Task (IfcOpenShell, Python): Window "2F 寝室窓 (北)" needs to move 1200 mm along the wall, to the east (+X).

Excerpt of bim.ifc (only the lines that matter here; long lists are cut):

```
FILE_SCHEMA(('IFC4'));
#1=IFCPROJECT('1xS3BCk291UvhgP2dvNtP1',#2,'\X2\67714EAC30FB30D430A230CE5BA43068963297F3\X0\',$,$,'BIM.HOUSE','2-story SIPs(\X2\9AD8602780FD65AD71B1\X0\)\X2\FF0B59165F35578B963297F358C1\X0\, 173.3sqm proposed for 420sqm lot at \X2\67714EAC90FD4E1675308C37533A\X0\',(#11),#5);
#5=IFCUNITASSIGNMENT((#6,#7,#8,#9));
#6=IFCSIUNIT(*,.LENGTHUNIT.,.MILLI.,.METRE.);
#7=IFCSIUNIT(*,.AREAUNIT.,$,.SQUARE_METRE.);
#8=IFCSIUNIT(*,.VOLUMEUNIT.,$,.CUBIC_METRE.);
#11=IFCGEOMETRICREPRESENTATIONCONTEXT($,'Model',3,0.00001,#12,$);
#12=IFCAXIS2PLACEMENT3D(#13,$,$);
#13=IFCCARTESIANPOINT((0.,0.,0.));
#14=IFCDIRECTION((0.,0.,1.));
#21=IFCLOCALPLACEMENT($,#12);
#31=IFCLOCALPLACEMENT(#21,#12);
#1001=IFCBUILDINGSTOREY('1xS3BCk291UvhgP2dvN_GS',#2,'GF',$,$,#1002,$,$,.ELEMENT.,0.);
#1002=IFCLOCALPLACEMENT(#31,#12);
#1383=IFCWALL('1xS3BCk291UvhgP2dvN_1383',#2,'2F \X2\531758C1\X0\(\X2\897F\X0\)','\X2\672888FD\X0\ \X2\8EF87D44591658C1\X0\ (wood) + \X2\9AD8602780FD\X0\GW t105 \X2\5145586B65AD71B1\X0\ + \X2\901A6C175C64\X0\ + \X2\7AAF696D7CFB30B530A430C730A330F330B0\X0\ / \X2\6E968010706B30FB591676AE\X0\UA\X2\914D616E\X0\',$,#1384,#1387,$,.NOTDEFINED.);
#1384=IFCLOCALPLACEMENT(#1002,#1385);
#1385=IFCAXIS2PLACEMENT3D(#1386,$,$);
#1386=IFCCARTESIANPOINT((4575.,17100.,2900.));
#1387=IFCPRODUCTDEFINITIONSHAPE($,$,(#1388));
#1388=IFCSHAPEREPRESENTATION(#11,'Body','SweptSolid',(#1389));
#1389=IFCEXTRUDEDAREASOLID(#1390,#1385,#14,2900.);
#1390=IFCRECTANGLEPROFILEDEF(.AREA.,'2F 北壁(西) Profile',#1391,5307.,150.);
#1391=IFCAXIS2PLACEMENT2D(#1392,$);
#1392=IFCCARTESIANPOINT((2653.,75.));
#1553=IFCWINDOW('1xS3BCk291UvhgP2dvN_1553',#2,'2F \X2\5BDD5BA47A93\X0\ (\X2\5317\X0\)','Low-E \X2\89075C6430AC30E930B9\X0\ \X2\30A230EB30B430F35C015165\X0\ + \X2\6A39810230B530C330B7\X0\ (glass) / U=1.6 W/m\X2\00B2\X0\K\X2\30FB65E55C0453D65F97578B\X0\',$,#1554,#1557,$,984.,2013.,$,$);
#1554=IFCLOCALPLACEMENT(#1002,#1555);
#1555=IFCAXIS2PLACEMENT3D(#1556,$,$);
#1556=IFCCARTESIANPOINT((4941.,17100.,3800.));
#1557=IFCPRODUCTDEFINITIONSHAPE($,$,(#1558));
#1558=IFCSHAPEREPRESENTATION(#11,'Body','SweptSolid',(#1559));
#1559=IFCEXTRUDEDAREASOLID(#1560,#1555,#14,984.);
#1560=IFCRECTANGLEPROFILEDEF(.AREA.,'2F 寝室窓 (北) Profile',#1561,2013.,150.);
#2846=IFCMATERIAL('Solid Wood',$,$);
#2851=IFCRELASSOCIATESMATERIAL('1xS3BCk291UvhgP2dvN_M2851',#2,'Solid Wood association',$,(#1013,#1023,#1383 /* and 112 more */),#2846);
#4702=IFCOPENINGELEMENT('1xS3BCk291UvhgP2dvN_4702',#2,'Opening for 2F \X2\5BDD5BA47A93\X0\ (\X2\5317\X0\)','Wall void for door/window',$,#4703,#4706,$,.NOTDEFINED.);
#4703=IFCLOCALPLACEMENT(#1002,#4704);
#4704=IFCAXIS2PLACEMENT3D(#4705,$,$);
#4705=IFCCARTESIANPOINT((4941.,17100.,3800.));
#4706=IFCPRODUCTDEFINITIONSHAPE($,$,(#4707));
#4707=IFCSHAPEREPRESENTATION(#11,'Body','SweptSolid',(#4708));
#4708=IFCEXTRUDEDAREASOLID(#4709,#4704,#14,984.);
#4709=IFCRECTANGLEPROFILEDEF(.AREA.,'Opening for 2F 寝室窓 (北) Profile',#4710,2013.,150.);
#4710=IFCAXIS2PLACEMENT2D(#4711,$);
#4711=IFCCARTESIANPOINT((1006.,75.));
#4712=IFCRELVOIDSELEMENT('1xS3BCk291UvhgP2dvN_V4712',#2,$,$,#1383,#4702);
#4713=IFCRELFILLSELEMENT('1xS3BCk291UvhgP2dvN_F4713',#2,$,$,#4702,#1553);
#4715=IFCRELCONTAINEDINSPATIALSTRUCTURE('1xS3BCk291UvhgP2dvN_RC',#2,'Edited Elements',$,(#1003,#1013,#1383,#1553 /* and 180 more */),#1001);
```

```python
import ifcopenshell
import ifcopenshell.api.geometry
import ifcopenshell.util.placement
import ifcopenshell.util.unit

model = ifcopenshell.open("bim.ifc")
unit_scale = ifcopenshell.util.unit.calculate_unit_scale(model)

window = model.by_id(1553)
opening = window.FillsVoids[0].RelatingOpeningElement
wall = opening.VoidsElements[0].RelatingBuildingElement

wall_matrix = ifcopenshell.util.placement.get_local_placement(wall.ObjectPlacement)
shift = wall_matrix[:3, 0] * 1.2 / unit_scale
before = ifcopenshell.util.placement.get_local_placement(window.ObjectPlacement)[:3, 3].copy()

# The window is not placed relative to its opening, so move both.
for product in (opening, window):
    matrix = ifcopenshell.util.placement.get_local_placement(product.ObjectPlacement)
    matrix[:3, 3] += shift
    ifcopenshell.api.geometry.edit_object_placement(model, product=product, matrix=matrix, is_si=False)

after = ifcopenshell.util.placement.get_local_placement(window.ObjectPlacement)[:3, 3]
print("window moved by", (after - before).round(3) + 0.0)

model.write("bim_rev.ifc")
```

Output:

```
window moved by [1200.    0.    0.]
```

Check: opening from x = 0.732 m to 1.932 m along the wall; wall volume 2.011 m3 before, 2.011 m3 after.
